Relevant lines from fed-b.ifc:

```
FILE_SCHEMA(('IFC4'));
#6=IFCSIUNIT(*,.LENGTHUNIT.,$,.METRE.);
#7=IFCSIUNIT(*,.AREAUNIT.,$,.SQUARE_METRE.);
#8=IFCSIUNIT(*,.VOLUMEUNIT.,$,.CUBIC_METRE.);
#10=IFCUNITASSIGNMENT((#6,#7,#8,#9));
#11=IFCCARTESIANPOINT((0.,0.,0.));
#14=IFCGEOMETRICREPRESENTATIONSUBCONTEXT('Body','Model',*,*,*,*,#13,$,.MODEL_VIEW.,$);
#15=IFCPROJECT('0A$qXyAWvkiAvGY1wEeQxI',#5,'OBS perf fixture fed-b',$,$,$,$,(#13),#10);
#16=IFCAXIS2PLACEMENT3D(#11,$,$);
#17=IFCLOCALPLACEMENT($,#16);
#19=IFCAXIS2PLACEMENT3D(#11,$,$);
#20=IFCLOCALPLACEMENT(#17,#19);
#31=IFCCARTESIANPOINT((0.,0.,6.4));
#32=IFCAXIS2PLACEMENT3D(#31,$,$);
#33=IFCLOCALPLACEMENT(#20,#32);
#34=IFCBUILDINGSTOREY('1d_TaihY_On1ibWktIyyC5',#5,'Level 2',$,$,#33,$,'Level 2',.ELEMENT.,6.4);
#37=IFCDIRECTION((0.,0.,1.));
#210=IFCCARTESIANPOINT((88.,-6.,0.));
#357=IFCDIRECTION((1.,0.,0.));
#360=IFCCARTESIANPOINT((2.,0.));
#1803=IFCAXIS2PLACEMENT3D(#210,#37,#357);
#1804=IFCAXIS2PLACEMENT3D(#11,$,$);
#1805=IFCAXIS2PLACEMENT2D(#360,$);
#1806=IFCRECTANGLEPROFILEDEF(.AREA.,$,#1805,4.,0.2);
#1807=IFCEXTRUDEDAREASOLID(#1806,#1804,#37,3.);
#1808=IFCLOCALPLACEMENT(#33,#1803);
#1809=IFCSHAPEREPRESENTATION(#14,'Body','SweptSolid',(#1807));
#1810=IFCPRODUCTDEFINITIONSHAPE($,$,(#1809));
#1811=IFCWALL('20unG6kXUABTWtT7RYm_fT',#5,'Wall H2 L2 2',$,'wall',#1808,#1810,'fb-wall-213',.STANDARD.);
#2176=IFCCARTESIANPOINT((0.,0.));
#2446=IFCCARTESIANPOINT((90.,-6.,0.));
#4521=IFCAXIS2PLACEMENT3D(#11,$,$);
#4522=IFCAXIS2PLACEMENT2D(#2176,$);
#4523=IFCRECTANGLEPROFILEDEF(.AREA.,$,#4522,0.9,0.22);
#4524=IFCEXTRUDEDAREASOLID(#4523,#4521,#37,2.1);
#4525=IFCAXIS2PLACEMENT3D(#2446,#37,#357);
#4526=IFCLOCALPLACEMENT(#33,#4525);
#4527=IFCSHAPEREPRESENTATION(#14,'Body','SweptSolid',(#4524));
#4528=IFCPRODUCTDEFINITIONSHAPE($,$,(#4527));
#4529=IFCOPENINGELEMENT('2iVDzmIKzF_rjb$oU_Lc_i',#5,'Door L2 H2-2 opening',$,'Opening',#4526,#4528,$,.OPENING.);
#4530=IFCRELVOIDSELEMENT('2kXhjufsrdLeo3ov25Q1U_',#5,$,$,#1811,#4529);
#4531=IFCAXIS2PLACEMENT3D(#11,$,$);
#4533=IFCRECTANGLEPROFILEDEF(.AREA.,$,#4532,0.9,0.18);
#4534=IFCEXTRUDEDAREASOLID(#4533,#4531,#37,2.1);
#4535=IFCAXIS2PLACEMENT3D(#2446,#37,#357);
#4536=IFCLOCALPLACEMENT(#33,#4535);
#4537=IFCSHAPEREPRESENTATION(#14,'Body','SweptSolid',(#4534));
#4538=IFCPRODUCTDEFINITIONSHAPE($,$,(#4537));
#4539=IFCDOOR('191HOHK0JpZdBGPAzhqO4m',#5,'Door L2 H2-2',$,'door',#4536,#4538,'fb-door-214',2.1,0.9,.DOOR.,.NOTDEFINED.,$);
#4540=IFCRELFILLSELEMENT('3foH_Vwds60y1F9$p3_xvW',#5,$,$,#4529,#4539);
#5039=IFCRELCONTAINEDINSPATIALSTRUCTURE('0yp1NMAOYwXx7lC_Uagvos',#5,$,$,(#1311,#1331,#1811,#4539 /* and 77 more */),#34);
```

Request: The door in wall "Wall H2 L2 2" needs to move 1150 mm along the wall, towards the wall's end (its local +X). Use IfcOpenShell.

```python
import ifcopenshell
import ifcopenshell.api.geometry
import ifcopenshell.util.placement

model = ifcopenshell.open("fed-b.ifc")

door = model.by_guid("191HOHK0JpZdBGPAzhqO4m")
opening = door.FillsVoids[0].RelatingOpeningElement
wall = opening.VoidsElements[0].RelatingBuildingElement

wall_matrix = ifcopenshell.util.placement.get_local_placement(wall.ObjectPlacement)
shift = wall_matrix[:3, 0] * 1.15
before = ifcopenshell.util.placement.get_local_placement(door.ObjectPlacement)[:3, 3].copy()

# The door is not placed relative to its opening, so move both.
for product in (opening, door):
    matrix = ifcopenshell.util.placement.get_local_placement(product.ObjectPlacement)
    matrix[:3, 3] += shift
    ifcopenshell.api.geometry.edit_object_placement(model, product=product, matrix=matrix, is_si=False)

after = ifcopenshell.util.placement.get_local_placement(door.ObjectPlacement)[:3, 3]
print("door moved by", (after - before).round(3) + 0.0)

model.write("fed-b_updated.ifc")
```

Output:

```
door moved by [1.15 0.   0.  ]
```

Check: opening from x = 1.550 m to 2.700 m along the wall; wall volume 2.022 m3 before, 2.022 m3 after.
